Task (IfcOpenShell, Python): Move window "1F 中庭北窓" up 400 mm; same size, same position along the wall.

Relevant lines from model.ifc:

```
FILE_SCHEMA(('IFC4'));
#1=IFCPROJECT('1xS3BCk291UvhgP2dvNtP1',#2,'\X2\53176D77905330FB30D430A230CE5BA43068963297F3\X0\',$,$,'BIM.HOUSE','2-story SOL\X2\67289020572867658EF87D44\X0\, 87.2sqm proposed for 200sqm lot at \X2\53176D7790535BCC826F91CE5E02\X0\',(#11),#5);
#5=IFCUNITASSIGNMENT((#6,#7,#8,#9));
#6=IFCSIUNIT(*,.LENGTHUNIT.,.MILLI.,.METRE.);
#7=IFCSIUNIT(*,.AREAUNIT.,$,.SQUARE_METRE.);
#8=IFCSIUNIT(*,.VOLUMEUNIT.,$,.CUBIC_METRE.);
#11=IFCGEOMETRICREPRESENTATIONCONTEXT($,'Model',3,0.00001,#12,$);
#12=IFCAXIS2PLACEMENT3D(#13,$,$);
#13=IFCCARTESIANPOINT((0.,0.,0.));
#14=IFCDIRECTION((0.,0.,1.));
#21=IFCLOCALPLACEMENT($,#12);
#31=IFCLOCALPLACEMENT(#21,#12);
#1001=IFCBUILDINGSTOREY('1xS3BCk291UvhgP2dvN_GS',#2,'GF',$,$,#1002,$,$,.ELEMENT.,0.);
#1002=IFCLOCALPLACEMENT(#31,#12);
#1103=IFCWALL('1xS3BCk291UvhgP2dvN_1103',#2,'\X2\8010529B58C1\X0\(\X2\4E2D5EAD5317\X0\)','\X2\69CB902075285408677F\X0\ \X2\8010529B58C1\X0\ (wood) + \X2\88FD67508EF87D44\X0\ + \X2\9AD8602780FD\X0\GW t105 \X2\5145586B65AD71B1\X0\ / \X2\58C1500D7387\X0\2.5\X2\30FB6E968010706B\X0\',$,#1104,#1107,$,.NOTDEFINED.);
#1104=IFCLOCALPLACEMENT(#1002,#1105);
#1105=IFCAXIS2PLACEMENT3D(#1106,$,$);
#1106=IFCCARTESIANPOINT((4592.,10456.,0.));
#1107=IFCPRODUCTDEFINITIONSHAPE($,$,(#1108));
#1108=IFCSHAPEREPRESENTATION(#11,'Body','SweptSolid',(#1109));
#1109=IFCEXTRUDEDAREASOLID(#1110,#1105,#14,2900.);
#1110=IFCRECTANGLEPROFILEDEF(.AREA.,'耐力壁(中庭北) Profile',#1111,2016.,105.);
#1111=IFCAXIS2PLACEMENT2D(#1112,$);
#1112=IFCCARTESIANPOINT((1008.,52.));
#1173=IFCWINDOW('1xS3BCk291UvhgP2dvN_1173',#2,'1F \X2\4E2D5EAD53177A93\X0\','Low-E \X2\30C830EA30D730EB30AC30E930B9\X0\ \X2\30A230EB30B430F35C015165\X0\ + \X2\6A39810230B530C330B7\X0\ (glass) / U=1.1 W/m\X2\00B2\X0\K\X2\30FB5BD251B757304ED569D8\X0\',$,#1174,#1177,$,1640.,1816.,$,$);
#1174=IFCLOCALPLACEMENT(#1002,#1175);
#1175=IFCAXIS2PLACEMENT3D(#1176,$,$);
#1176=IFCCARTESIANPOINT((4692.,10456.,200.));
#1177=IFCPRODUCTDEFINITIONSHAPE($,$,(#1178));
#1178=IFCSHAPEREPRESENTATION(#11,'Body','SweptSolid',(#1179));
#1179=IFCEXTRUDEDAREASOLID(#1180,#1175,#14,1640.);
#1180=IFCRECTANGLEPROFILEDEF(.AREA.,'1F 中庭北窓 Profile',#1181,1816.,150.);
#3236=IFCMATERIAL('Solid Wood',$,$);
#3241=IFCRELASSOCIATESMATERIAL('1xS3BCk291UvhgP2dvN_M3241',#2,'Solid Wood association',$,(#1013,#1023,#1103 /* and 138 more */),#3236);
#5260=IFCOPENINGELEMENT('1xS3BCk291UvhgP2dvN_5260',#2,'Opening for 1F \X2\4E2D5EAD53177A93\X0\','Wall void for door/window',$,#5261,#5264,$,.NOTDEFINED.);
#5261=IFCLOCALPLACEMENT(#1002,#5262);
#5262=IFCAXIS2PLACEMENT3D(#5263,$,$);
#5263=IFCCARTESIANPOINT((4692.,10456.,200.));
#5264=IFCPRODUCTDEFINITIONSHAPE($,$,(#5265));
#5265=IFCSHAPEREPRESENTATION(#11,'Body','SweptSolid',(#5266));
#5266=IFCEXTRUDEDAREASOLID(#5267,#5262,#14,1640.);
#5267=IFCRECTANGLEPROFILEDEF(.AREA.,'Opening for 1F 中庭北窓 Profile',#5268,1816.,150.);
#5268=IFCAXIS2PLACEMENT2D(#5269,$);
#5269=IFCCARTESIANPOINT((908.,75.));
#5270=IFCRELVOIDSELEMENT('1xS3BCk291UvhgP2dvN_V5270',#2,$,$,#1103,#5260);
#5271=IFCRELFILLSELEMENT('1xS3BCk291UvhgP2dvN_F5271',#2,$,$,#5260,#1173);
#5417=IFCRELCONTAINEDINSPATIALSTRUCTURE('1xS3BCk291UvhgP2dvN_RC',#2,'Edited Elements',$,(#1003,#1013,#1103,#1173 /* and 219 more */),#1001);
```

```python
import numpy as np
import ifcopenshell
import ifcopenshell.api.geometry
import ifcopenshell.util.placement
import ifcopenshell.util.unit

model = ifcopenshell.open("model.ifc")
unit_scale = ifcopenshell.util.unit.calculate_unit_scale(model)

window = model.by_id(1173)
opening = window.FillsVoids[0].RelatingOpeningElement
dz = 400.0

shift = np.array([0.0, 0.0, dz])
# The window is not placed relative to its opening, so move both.
for product in (opening, window):
    matrix = ifcopenshell.util.placement.get_local_placement(product.ObjectPlacement)
    matrix[:3, 3] += shift
    ifcopenshell.api.geometry.edit_object_placement(model, product=product, matrix=matrix, is_si=False)

print(f"moved by {dz * unit_scale:+.3f} m")

model.write("model-out.ifc")
```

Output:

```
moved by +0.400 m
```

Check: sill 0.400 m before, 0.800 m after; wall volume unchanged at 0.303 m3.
